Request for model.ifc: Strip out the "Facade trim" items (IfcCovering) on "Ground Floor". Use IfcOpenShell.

First a look at what the model holds.

```python
import ifcopenshell
import ifcopenshell.util.element

model = ifcopenshell.open("model.ifc")
print(model.schema)
storey = next(s for s in model.by_type("IfcBuildingStorey") if s.Name == "Ground Floor")
coverings = [e for e in ifcopenshell.util.element.get_decomposition(storey) if e.is_a("IfcCovering")]
seen = {}
for e in coverings:
    element_type = ifcopenshell.util.element.get_type(e)
    name = element_type.Name if element_type not in (None, e) else None
    seen[name] = seen.get(name, 0) + 1
for name, count in sorted(seen.items(), key=str):
    print(count, "x", name)
```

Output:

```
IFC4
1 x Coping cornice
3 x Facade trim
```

```python
import ifcopenshell
import ifcopenshell.api.root
import ifcopenshell.util.element

model = ifcopenshell.open("model.ifc")

storey = next(s for s in model.by_type("IfcBuildingStorey") if s.Name == "Ground Floor")
coverings = [e for e in ifcopenshell.util.element.get_decomposition(storey) if e.is_a("IfcCovering")]
targets = [e for e in coverings if (t := ifcopenshell.util.element.get_type(e)) not in (None, e) and t.Name == "Facade trim"]

for e in targets:
    ifcopenshell.api.root.remove_product(model, product=e)
print(len(targets), "removed")

model.write("model_rev.ifc")
```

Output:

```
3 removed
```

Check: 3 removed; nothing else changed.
